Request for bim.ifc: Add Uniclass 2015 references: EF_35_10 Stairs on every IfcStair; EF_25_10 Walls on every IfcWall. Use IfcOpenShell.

First a look at what the model holds.

```python
import ifcopenshell

model = ifcopenshell.open("bim.ifc")
print(model.schema)
print("classifications:", [c.Name for c in model.by_type("IfcClassification")])
for ifc_class in ("IfcDoor", "IfcRoof", "IfcStair", "IfcWall", "IfcWindow"):
    print(ifc_class, len(model.by_type(ifc_class)))
```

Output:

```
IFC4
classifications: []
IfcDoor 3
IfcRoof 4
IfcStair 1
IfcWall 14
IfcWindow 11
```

```python
import ifcopenshell
import ifcopenshell.api.classification

model = ifcopenshell.open("bim.ifc")

system = ifcopenshell.api.classification.add_classification(model, classification="Uniclass 2015")

codes = {
    "IfcStair": ("EF_35_10", "Stairs"),
    "IfcWall": ("EF_25_10", "Walls"),
}
for ifc_class, (code, name) in codes.items():
    products = model.by_type(ifc_class)
    ifcopenshell.api.classification.add_reference(
        model, products=products, classification=system, identification=code, name=name
    )
    print(code, len(products))

model.write("bim_updated.ifc")
```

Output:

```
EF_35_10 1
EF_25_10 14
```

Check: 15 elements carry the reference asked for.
